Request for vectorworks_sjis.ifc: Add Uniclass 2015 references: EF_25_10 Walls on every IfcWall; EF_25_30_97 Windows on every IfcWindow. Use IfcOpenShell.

First a look at what the model holds.

```python
import ifcopenshell

model = ifcopenshell.open("vectorworks_sjis.ifc")
print(model.schema)
print("classifications:", [c.Name for c in model.by_type("IfcClassification")])
for ifc_class in ("IfcDoor", "IfcRoof", "IfcStair", "IfcWall", "IfcWindow"):
    print(ifc_class, len(model.by_type(ifc_class)))
```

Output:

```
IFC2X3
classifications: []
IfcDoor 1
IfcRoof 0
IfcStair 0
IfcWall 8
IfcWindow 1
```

```python
import ifcopenshell
import ifcopenshell.api.classification

model = ifcopenshell.open("vectorworks_sjis.ifc")

# IFC2X3 requires Source and Edition and has no link from the project to the system.
system = model.create_entity("IfcClassification", Source="NBS", Edition="2015", Name="Uniclass 2015")

codes = {
    "IfcWall": ("EF_25_10", "Walls"),
    "IfcWindow": ("EF_25_30_97", "Windows"),
}
for ifc_class, (code, name) in codes.items():
    products = model.by_type(ifc_class)
    ifcopenshell.api.classification.add_reference(
        model, products=products, classification=system, identification=code, name=name
    )
    print(code, len(products))

model.write("vectorworks_sjis_updated.ifc")
```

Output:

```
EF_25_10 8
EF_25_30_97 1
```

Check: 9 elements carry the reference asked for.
